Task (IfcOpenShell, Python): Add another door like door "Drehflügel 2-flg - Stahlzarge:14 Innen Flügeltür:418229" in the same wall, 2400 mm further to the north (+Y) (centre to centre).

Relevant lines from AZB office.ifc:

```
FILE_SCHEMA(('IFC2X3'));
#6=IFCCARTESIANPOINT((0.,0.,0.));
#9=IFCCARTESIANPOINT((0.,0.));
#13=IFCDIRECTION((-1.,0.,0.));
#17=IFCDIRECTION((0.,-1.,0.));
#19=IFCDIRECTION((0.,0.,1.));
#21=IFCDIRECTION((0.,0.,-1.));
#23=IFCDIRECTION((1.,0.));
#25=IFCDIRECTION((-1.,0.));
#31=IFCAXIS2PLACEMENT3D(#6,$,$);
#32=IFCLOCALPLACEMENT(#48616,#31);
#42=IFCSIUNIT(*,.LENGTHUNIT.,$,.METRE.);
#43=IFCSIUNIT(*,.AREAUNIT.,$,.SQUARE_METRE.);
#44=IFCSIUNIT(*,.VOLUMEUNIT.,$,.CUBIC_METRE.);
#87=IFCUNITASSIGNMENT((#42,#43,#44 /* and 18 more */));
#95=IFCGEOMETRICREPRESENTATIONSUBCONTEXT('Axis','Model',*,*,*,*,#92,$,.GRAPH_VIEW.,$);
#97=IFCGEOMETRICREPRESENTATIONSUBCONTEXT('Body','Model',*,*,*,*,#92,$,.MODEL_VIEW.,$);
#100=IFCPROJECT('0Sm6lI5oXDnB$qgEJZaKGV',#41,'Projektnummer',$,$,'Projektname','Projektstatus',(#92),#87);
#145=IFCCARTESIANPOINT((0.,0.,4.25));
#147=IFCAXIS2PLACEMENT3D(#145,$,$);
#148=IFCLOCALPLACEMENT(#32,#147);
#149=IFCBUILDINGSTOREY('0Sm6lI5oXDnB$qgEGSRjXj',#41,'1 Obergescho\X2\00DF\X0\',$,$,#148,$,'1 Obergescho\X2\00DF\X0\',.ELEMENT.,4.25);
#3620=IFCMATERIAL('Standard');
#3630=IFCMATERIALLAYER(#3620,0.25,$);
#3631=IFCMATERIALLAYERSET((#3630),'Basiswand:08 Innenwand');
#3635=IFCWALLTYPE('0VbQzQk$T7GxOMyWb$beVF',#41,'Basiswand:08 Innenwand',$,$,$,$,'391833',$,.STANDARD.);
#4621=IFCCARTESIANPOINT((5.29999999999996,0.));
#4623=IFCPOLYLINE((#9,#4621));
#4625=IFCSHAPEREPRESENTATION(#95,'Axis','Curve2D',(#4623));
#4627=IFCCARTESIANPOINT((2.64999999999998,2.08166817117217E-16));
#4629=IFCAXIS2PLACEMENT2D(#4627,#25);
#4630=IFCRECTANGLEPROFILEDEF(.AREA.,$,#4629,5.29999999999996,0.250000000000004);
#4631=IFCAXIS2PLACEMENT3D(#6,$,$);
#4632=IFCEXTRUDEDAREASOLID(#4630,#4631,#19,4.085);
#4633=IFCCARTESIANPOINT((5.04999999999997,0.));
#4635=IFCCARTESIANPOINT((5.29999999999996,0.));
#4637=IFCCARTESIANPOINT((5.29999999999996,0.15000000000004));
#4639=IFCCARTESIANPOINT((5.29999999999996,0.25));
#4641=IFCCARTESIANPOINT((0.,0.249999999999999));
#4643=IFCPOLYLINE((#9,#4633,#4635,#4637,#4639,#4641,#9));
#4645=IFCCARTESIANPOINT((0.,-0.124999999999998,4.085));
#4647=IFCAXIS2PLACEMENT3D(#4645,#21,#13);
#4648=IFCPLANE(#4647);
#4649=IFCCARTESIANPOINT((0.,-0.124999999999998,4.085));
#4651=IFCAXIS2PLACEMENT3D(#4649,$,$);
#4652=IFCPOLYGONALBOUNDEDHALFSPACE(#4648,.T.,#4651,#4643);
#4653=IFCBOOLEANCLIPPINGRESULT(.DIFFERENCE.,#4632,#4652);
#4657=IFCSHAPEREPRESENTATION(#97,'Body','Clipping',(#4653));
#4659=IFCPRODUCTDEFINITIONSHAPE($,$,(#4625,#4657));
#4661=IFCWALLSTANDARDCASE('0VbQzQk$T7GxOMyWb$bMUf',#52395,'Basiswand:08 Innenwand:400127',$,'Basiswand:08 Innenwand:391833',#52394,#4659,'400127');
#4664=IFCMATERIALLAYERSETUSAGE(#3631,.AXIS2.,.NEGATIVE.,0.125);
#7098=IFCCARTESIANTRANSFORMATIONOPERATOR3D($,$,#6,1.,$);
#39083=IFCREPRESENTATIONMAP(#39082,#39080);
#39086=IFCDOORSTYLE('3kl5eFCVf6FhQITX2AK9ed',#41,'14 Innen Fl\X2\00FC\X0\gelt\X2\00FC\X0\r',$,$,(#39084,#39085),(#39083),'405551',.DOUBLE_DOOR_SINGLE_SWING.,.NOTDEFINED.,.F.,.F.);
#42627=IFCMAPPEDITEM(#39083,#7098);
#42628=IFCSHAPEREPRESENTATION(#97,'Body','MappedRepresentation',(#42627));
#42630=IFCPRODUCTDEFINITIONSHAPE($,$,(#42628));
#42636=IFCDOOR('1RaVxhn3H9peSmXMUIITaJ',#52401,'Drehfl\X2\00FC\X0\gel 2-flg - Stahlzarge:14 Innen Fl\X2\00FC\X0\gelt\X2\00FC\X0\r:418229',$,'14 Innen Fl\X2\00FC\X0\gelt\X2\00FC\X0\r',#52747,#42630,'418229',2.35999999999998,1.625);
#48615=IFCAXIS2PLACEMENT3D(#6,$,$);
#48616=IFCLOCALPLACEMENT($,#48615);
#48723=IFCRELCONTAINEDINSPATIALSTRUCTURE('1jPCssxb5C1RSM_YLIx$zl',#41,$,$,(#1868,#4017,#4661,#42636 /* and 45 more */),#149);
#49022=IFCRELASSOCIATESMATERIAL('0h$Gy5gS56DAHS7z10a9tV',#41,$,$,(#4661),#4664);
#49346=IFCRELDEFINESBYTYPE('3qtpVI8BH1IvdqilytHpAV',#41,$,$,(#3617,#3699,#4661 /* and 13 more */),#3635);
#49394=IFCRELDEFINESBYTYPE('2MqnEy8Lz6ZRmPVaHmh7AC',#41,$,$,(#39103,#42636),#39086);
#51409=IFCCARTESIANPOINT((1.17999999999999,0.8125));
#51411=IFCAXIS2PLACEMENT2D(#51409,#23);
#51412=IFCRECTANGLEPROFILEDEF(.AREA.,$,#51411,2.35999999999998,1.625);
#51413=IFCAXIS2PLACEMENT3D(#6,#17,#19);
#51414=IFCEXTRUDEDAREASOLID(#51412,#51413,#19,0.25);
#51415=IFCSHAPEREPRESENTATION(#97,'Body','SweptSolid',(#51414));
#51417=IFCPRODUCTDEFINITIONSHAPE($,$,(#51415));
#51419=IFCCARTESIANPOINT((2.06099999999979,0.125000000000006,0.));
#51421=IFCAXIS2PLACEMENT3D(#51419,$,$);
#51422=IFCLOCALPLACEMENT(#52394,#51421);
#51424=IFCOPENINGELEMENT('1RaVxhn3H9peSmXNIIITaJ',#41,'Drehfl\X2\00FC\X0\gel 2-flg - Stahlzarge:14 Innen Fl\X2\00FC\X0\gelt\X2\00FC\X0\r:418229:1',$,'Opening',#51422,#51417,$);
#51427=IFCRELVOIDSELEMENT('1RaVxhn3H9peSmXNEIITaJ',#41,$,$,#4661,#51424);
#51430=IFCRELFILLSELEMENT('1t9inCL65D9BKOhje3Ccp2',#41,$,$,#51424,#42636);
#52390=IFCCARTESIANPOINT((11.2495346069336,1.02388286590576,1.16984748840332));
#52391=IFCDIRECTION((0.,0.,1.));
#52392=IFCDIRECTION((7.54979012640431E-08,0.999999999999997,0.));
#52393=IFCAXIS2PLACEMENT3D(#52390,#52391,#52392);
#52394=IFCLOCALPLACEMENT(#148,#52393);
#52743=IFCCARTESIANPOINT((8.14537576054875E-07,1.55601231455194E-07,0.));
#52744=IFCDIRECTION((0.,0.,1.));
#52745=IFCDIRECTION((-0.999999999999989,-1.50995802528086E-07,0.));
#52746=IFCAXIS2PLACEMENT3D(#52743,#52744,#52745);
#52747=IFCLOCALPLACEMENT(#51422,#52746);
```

```python
import ifcopenshell
import ifcopenshell.api.feature
import ifcopenshell.api.geometry
import ifcopenshell.api.root
import ifcopenshell.geom
import ifcopenshell.util.element
import ifcopenshell.util.placement
import ifcopenshell.util.shape

model = ifcopenshell.open("AZB office.ifc")
settings = ifcopenshell.geom.settings()


def volume(element):
    """Net volume in cubic metres, openings subtracted."""
    shape = ifcopenshell.geom.create_shape(settings, element)
    return ifcopenshell.util.shape.get_volume(shape.geometry)


def reuse_history(source, copy):
    """copy_class also copies each property set's owner history, people and application; keep the originals."""
    for rel in copy.IsDefinedBy:
        if rel.is_a("IfcRelDefinesByProperties") and (history := rel.RelatingPropertyDefinition.OwnerHistory):
            rel.RelatingPropertyDefinition.OwnerHistory = source.OwnerHistory
            ifcopenshell.util.element.remove_deep2(model, history)


door = model.by_guid("1RaVxhn3H9peSmXMUIITaJ")
opening = door.FillsVoids[0].RelatingOpeningElement
wall = opening.VoidsElements[0].RelatingBuildingElement
before = volume(wall)
shift = ifcopenshell.util.placement.get_local_placement(wall.ObjectPlacement)[:3, 0] * 2.4

# copy_class copies the void relationship, type, container and properties, but no geometry.
new_opening = ifcopenshell.api.root.copy_class(model, product=opening)
new_opening.Representation = ifcopenshell.util.element.copy_deep(
    model, opening.Representation, exclude=["IfcGeometricRepresentationContext", "IfcRepresentationMap"]
)
new_opening.Name = "Drehflügel 2-flg - Stahlzarge:14 Innen Flügeltür"
new_door = ifcopenshell.api.root.copy_class(model, product=door)
new_door.Representation = ifcopenshell.util.element.copy_deep(
    model, door.Representation, exclude=["IfcGeometricRepresentationContext", "IfcRepresentationMap"]
)
new_door.Name = "Drehflügel 2-flg - Stahlzarge:14 Innen Flügeltür"
new_door.Tag = None
reuse_history(door, new_door)
fills = ifcopenshell.api.feature.add_filling(model, opening=new_opening, element=new_door)
fills.OwnerHistory = new_door.OwnerHistory  # required in IFC2X3

for old, new in ((opening, new_opening), (door, new_door)):
    matrix = ifcopenshell.util.placement.get_local_placement(old.ObjectPlacement)
    matrix[:3, 3] += shift
    ifcopenshell.api.geometry.edit_object_placement(model, product=new, matrix=matrix, is_si=False)

after = volume(wall)

print(f"wall volume {before:.3f} -> {after:.3f} m3")

model.write("AZB office_v2.ifc")
```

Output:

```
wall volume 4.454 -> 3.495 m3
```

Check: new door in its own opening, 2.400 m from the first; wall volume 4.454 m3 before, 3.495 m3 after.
